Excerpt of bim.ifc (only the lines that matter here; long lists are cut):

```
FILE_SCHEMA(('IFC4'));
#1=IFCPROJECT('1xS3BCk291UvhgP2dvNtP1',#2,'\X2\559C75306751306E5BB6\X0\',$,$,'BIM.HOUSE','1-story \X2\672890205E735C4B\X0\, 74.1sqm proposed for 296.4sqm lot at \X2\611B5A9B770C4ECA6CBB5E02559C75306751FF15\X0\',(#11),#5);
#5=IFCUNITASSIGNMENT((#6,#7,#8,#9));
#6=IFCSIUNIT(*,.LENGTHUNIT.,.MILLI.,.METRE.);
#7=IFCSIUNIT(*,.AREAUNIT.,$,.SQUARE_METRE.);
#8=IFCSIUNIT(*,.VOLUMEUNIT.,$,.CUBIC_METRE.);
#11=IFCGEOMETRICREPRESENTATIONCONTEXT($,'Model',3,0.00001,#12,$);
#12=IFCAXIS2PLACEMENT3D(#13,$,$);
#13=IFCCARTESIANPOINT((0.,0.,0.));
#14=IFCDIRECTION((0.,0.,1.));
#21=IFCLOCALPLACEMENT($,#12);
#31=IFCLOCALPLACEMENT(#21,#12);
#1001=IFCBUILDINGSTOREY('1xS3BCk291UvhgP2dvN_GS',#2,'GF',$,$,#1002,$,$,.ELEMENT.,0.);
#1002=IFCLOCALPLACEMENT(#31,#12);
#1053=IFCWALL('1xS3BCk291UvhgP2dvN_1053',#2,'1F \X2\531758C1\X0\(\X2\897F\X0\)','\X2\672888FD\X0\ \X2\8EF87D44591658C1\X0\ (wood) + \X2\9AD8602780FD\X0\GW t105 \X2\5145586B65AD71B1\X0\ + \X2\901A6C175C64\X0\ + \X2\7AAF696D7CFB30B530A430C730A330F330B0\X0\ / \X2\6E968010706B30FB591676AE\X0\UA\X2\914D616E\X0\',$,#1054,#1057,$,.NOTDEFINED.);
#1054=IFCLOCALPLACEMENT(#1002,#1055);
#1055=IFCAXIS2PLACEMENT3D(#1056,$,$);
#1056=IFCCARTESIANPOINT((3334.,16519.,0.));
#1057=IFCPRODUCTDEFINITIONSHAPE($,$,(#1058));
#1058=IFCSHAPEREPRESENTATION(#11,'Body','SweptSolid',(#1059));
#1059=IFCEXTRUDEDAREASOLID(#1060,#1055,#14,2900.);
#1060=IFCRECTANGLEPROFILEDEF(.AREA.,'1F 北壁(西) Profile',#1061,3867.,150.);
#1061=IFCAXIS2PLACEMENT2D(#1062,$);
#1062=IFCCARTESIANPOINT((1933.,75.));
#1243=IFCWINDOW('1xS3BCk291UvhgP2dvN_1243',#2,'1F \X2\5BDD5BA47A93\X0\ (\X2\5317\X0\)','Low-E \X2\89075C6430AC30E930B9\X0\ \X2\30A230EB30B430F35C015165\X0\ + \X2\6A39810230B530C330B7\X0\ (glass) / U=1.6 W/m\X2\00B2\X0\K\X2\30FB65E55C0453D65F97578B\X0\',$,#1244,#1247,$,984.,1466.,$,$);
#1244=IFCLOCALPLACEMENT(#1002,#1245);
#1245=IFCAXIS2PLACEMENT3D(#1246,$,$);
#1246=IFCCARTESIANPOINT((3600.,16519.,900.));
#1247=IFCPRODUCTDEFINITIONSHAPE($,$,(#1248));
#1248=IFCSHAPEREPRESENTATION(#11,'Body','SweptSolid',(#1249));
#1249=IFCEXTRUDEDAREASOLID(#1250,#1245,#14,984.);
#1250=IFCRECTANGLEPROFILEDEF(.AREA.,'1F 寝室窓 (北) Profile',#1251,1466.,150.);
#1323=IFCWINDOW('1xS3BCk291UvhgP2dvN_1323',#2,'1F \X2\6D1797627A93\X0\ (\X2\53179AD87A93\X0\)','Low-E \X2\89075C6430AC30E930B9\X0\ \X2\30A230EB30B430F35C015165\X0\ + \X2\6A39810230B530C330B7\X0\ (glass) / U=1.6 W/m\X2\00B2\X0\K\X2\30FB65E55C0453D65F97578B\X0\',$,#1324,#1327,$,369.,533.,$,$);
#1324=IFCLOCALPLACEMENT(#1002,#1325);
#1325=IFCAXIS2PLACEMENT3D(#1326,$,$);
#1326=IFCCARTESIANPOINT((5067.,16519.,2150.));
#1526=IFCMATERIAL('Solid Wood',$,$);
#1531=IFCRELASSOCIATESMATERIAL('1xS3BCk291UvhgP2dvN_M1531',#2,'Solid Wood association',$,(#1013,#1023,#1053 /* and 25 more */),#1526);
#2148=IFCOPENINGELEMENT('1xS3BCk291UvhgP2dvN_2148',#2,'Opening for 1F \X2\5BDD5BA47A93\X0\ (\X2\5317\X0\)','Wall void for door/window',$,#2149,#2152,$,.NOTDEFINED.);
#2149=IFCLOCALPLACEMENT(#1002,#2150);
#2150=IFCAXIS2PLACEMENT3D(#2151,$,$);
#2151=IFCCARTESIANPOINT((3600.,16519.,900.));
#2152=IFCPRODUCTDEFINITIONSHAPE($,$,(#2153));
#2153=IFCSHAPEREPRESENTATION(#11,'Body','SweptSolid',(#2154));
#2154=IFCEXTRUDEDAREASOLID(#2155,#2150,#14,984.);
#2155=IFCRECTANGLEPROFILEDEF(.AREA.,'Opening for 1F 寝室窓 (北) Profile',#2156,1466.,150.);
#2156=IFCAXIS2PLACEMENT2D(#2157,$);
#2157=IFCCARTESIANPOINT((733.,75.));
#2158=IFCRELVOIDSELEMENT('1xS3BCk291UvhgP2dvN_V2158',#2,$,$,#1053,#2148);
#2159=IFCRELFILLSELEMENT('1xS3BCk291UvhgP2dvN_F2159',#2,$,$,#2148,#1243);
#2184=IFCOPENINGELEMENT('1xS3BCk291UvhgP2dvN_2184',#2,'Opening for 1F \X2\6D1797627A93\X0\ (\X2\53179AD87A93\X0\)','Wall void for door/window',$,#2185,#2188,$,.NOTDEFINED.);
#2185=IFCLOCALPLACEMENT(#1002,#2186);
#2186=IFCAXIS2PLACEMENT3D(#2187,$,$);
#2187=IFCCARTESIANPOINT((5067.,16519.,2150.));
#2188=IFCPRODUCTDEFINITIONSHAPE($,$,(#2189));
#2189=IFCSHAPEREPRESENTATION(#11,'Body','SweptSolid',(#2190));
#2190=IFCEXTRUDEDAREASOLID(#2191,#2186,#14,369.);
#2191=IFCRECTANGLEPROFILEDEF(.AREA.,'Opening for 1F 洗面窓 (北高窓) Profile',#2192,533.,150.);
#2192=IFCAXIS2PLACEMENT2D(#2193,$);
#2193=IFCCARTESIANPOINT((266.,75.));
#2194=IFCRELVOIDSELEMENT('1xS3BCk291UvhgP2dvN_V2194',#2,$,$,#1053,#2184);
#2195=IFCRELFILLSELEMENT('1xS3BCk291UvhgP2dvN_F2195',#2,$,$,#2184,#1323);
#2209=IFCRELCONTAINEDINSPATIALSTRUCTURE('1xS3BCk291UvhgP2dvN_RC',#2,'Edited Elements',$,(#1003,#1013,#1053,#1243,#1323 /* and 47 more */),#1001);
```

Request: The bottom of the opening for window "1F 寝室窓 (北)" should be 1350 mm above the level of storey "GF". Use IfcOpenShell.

```python
import numpy as np
import ifcopenshell
import ifcopenshell.api.geometry
import ifcopenshell.geom
import ifcopenshell.util.element
import ifcopenshell.util.placement
import ifcopenshell.util.shape
import ifcopenshell.util.unit

model = ifcopenshell.open("bim.ifc")
unit_scale = ifcopenshell.util.unit.calculate_unit_scale(model)

window = model.by_id(1243)
opening = window.FillsVoids[0].RelatingOpeningElement
storey = ifcopenshell.util.element.get_container(window, ifc_class="IfcBuildingStorey")
level = ifcopenshell.util.placement.get_local_placement(storey.ObjectPlacement)[2, 3]

# The opening's origin need not be at the sill, so measure its lowest point.
shape = ifcopenshell.geom.create_shape(ifcopenshell.geom.settings(), opening)
bottom = ifcopenshell.util.shape.get_shape_bottom_elevation(shape, shape.geometry) / unit_scale
dz = level + 1.35 / unit_scale - bottom

shift = np.array([0.0, 0.0, dz])
# The window is not placed relative to its opening, so move both.
for product in (opening, window):
    matrix = ifcopenshell.util.placement.get_local_placement(product.ObjectPlacement)
    matrix[:3, 3] += shift
    ifcopenshell.api.geometry.edit_object_placement(model, product=product, matrix=matrix, is_si=False)

print(f"moved by {dz * unit_scale:+.3f} m")

model.write("bim_rev.ifc")
```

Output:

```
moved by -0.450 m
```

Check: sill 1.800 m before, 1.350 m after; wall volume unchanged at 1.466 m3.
